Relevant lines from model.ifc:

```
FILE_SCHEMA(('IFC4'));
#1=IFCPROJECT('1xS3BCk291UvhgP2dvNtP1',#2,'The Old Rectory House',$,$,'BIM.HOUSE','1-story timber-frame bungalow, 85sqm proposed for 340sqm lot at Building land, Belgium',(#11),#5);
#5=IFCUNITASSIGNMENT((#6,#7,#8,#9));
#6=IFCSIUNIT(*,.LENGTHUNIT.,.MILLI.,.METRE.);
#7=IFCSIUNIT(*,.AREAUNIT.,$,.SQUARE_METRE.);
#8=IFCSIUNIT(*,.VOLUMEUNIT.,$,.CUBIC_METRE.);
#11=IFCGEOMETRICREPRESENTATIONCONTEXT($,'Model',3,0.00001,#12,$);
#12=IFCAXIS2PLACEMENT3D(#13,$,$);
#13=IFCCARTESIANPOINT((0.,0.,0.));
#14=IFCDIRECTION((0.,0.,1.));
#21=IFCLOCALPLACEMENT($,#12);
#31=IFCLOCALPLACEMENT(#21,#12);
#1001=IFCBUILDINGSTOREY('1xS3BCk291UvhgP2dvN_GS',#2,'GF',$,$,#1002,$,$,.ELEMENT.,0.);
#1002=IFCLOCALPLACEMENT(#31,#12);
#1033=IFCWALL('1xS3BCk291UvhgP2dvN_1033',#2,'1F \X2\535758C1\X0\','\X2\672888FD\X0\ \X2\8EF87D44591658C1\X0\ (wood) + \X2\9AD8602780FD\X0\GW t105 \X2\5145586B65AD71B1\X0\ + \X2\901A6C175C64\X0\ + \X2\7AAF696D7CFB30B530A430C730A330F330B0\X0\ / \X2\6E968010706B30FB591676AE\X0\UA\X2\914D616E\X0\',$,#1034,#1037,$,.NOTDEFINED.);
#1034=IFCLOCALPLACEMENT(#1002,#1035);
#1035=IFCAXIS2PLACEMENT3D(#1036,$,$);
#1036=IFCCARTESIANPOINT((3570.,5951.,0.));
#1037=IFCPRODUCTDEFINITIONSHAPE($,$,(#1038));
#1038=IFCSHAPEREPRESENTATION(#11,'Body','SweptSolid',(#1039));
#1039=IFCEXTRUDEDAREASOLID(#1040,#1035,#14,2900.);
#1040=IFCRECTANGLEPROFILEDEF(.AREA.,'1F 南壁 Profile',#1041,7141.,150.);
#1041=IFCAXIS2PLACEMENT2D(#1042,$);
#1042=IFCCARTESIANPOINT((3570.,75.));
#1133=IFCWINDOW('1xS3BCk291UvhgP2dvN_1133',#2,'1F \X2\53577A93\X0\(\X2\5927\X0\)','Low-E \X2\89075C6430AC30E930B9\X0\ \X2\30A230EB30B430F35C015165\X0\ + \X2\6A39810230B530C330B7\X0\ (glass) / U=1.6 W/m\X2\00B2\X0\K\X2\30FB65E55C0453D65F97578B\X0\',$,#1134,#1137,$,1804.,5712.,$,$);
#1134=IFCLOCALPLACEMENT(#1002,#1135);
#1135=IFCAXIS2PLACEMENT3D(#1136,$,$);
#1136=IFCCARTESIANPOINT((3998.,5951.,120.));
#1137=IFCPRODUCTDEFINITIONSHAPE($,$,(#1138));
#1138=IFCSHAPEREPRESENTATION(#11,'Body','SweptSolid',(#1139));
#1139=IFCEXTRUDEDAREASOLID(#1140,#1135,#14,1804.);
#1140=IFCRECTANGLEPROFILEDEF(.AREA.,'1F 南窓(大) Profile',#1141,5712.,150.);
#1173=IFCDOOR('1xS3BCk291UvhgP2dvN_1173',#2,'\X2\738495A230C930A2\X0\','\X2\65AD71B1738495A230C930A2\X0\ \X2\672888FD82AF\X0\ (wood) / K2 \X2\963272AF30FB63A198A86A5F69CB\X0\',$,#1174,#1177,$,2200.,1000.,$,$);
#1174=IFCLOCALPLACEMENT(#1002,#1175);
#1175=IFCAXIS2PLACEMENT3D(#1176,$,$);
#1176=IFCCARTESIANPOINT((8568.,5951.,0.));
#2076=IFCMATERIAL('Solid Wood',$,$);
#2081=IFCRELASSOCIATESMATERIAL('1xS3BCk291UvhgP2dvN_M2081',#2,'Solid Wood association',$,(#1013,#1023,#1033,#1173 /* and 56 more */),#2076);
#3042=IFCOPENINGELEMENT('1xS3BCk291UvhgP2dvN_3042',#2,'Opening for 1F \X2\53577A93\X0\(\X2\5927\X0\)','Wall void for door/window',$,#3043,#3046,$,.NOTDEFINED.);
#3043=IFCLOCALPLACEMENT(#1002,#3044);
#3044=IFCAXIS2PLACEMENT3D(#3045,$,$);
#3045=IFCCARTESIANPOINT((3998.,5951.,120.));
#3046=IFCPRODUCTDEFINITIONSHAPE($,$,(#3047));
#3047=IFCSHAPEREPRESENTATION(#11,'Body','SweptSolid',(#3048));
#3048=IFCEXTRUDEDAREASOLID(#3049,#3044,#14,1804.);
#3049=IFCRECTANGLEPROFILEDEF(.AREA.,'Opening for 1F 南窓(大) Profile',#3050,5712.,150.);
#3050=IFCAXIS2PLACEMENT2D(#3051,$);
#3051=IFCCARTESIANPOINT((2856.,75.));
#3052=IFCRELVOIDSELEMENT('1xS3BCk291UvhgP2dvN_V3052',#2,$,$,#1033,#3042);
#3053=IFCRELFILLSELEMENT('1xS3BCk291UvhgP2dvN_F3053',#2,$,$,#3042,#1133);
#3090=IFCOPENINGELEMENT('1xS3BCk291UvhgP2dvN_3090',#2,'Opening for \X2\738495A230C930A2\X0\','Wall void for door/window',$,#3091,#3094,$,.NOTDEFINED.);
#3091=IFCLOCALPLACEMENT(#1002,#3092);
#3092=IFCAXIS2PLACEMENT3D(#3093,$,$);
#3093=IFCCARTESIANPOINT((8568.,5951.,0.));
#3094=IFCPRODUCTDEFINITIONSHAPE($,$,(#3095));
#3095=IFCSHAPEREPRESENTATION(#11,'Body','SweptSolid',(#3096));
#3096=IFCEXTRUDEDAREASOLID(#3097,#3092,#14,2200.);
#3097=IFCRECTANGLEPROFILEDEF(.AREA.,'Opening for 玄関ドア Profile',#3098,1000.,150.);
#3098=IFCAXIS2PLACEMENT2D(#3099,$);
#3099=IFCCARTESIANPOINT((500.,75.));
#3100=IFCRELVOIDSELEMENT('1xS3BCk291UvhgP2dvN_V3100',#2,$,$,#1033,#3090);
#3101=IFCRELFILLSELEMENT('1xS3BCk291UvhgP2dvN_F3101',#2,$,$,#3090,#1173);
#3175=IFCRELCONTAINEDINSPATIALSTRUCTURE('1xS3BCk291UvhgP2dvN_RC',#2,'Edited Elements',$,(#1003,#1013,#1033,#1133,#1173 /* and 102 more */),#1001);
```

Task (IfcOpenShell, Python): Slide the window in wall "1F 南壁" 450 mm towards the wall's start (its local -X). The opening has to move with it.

```python
import ifcopenshell
import ifcopenshell.api.geometry
import ifcopenshell.util.placement
import ifcopenshell.util.unit

model = ifcopenshell.open("model.ifc")
unit_scale = ifcopenshell.util.unit.calculate_unit_scale(model)

window = model.by_guid("1xS3BCk291UvhgP2dvN_1133")
opening = window.FillsVoids[0].RelatingOpeningElement
wall = opening.VoidsElements[0].RelatingBuildingElement

wall_matrix = ifcopenshell.util.placement.get_local_placement(wall.ObjectPlacement)
shift = wall_matrix[:3, 0] * -0.45 / unit_scale
before = ifcopenshell.util.placement.get_local_placement(window.ObjectPlacement)[:3, 3].copy()

# The window is not placed relative to its opening, so move both.
for product in (opening, window):
    matrix = ifcopenshell.util.placement.get_local_placement(product.ObjectPlacement)
    matrix[:3, 3] += shift
    ifcopenshell.api.geometry.edit_object_placement(model, product=product, matrix=matrix, is_si=False)

after = ifcopenshell.util.placement.get_local_placement(window.ObjectPlacement)[:3, 3]
print("window moved by", (after - before).round(3) + 0.0)

model.write("model_rev.ifc")
```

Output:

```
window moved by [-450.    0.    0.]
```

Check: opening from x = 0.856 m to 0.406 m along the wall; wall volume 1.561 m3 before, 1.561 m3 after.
